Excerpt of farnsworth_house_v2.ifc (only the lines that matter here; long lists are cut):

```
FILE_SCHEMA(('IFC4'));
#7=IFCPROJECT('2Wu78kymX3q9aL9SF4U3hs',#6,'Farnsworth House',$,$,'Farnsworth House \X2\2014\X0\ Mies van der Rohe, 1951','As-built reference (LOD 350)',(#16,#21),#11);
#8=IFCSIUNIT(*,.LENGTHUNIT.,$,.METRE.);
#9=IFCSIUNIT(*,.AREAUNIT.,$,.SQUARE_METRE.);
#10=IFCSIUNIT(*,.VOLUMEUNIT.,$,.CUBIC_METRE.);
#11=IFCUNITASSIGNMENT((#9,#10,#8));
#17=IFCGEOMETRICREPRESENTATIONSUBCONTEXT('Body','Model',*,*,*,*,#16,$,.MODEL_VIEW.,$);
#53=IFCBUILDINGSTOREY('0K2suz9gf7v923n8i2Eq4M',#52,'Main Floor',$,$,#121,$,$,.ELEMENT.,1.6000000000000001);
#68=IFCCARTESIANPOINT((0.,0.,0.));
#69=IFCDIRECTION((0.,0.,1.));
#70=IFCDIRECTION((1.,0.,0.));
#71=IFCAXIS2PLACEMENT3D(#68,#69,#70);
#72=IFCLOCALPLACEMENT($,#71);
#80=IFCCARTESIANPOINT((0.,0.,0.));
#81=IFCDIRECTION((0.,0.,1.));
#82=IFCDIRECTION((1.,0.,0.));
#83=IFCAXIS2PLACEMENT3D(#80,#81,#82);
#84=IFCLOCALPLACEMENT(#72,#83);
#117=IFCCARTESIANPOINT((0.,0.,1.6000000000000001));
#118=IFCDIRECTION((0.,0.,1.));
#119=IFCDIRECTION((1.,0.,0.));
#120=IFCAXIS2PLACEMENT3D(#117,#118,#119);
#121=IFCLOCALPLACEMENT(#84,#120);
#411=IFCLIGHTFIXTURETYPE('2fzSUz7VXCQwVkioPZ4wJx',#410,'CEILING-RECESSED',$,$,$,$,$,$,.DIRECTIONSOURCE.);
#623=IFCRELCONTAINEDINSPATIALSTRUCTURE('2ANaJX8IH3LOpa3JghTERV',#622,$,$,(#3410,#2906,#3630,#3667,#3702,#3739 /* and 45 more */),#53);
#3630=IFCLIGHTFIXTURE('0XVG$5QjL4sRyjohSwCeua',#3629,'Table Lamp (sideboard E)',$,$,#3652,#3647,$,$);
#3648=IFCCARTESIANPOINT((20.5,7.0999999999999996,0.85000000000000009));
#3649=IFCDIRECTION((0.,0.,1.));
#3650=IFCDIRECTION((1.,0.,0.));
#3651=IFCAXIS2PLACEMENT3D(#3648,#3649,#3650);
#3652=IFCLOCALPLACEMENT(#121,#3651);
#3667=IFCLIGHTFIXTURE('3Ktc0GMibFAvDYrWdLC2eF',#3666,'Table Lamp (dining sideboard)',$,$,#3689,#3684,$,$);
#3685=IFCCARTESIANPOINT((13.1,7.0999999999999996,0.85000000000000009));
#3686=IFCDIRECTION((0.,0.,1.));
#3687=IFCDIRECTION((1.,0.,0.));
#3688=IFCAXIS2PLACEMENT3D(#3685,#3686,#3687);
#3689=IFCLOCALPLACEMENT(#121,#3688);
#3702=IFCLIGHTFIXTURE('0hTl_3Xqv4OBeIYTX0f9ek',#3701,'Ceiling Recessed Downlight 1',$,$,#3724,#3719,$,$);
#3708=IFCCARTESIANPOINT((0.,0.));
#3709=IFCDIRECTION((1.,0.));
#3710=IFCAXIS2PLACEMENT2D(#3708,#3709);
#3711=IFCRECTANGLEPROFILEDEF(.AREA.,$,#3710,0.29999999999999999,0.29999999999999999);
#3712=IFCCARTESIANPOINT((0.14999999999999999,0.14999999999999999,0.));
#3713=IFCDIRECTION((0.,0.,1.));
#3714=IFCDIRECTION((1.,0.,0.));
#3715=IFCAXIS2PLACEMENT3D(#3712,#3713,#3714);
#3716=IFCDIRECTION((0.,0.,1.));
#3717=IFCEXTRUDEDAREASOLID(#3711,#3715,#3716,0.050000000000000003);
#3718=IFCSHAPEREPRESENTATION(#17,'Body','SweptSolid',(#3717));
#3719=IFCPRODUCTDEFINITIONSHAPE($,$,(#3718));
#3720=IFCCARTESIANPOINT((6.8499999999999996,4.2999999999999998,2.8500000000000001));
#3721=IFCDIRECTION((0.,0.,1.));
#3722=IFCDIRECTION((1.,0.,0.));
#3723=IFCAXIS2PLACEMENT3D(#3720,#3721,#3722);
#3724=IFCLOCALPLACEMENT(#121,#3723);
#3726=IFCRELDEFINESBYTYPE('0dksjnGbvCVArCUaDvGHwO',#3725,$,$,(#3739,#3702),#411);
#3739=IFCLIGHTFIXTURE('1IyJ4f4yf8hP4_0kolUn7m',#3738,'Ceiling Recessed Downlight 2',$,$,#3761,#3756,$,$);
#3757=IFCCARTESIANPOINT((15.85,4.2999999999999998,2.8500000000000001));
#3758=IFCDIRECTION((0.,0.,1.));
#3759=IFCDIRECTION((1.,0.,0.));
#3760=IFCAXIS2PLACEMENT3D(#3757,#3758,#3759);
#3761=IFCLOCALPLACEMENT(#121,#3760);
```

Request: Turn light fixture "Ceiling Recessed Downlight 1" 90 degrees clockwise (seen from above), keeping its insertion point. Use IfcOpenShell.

```python
import ifcopenshell
import ifcopenshell.api.geometry
import ifcopenshell.util.placement

model = ifcopenshell.open("farnsworth_house_v2.ifc")

item = model.by_guid("0hTl_3Xqv4OBeIYTX0f9ek")
matrix = ifcopenshell.util.placement.get_local_placement(item.ObjectPlacement)
matrix = matrix @ ifcopenshell.util.placement.rotation(-90, "Z")
ifcopenshell.api.geometry.edit_object_placement(model, product=item, matrix=matrix, is_si=False)

print(ifcopenshell.util.placement.get_local_placement(item.ObjectPlacement).round(3) + 0.0)

model.write("farnsworth_house_v2_rev.ifc")
```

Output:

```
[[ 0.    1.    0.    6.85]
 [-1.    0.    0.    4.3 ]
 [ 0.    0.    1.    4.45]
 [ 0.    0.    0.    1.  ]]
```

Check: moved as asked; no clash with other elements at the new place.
